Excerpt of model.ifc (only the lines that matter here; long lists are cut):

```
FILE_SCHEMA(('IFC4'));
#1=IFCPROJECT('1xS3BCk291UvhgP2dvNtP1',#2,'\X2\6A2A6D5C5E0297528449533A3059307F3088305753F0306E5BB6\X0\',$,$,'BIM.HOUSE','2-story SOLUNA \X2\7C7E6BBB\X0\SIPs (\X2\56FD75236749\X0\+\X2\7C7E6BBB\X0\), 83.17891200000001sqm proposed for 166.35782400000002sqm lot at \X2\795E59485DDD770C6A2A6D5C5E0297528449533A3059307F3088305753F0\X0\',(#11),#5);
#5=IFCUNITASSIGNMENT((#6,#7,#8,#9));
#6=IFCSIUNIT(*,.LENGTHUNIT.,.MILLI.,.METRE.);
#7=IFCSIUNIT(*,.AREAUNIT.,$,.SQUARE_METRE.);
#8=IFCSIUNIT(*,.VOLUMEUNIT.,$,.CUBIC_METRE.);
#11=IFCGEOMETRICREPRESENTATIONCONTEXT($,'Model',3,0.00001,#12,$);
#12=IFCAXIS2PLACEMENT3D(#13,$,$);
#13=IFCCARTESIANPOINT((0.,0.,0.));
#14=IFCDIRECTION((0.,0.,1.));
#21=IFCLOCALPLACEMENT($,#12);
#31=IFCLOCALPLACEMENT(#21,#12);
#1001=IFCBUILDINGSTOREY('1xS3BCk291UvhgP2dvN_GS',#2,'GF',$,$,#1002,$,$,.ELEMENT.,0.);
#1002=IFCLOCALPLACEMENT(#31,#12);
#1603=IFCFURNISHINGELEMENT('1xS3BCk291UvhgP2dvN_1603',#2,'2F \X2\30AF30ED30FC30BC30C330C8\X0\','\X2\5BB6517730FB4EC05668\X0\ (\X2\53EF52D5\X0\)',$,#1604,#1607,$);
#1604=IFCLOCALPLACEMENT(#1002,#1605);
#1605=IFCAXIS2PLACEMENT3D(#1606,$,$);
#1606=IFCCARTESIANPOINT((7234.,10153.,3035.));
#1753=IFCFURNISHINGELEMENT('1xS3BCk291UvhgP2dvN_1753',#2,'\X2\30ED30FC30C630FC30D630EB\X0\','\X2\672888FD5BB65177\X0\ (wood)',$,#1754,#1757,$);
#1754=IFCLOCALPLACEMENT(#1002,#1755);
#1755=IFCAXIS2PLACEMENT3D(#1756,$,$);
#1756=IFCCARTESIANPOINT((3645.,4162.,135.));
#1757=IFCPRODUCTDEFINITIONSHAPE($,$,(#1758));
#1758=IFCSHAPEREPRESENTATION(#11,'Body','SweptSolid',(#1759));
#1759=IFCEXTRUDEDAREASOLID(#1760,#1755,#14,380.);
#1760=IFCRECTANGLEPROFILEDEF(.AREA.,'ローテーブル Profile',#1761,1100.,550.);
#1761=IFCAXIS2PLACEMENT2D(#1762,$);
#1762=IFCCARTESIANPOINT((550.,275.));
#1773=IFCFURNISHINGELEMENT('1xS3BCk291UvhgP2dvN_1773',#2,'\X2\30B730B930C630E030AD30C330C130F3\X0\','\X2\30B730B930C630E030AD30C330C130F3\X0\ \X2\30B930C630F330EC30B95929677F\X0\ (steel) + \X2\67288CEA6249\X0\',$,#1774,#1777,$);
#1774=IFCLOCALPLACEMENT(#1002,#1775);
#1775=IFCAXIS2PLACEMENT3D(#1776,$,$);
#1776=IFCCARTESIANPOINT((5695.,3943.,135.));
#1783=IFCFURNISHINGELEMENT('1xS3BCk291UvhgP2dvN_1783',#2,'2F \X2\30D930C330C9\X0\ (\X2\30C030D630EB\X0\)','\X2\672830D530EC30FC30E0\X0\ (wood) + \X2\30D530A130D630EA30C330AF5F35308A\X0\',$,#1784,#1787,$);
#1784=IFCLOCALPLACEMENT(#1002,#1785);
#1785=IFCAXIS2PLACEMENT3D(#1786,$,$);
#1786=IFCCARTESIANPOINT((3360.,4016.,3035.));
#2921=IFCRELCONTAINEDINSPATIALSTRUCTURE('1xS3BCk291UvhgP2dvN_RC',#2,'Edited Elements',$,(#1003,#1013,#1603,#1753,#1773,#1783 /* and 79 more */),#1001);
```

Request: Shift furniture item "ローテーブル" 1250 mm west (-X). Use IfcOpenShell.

```python
import ifcopenshell
import ifcopenshell.api.geometry
import ifcopenshell.util.placement
import ifcopenshell.util.unit

model = ifcopenshell.open("model.ifc")
unit_scale = ifcopenshell.util.unit.calculate_unit_scale(model)

item = model.by_guid("1xS3BCk291UvhgP2dvN_1753")
matrix = ifcopenshell.util.placement.get_local_placement(item.ObjectPlacement)
matrix[0, 3] -= 1.25 / unit_scale
ifcopenshell.api.geometry.edit_object_placement(model, product=item, matrix=matrix, is_si=False)

print(ifcopenshell.util.placement.get_local_placement(item.ObjectPlacement).round(3) + 0.0)

model.write("model_edited.ifc")
```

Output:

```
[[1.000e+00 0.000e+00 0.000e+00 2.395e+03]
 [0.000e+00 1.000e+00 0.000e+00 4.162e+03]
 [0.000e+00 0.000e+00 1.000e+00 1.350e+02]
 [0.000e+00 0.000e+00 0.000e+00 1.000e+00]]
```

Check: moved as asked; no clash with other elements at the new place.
